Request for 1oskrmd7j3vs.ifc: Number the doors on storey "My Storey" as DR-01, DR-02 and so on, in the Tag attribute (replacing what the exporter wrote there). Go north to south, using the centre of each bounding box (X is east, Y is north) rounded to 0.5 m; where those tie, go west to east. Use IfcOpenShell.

First a look at what the model holds.

```python
import ifcopenshell
import ifcopenshell.util.element
import ifcopenshell.util.placement

model = ifcopenshell.open("1oskrmd7j3vs.ifc")
print(model.schema)
storey = next(s for s in model.by_type("IfcBuildingStorey") if s.Name == "My Storey")
doors = [e for e in ifcopenshell.util.element.get_decomposition(storey) if e.is_a("IfcDoor")]
for e in sorted(doors, key=lambda e: e.id()):
    origin = ifcopenshell.util.placement.get_local_placement(e.ObjectPlacement)[:3, 3]
    print(e.id(), e.Tag, e.Name, origin.round(2) + 0.0, sep=" | ")
```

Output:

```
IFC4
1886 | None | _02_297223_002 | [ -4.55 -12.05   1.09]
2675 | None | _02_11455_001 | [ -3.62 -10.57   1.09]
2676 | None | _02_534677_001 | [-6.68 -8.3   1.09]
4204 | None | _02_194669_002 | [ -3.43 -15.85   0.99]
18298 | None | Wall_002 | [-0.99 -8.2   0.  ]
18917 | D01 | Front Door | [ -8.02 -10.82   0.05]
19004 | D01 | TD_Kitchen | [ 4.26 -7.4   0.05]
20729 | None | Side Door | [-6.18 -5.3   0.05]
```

```python
import ifcopenshell
import ifcopenshell.geom
import ifcopenshell.util.element
import ifcopenshell.util.shape

model = ifcopenshell.open("1oskrmd7j3vs.ifc")
settings = ifcopenshell.geom.settings()
settings.set("use-world-coords", True)


def centre(element):
    shape = ifcopenshell.geom.create_shape(settings, element)
    return ifcopenshell.util.shape.get_bbox_centroid(shape.geometry)


storey = next(s for s in model.by_type("IfcBuildingStorey") if s.Name == "My Storey")
doors = [e for e in ifcopenshell.util.element.get_decomposition(storey) if e.is_a("IfcDoor")]

# Insertion points can sit at a corner or the storey origin, so sort by the geometry (in metres).
centres = {e: centre(e) for e in doors}
doors.sort(key=lambda e: (-round(centres[e][1] / 0.5), centres[e][0]))

for i, e in enumerate(doors, start=1):
    number = f"DR-{i:02d}"
    e.Tag = number
    print(e.id(), number)

model.write("1oskrmd7j3vs_edited.ifc")
```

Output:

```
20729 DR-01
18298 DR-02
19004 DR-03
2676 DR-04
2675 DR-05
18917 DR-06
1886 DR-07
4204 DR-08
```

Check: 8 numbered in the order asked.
